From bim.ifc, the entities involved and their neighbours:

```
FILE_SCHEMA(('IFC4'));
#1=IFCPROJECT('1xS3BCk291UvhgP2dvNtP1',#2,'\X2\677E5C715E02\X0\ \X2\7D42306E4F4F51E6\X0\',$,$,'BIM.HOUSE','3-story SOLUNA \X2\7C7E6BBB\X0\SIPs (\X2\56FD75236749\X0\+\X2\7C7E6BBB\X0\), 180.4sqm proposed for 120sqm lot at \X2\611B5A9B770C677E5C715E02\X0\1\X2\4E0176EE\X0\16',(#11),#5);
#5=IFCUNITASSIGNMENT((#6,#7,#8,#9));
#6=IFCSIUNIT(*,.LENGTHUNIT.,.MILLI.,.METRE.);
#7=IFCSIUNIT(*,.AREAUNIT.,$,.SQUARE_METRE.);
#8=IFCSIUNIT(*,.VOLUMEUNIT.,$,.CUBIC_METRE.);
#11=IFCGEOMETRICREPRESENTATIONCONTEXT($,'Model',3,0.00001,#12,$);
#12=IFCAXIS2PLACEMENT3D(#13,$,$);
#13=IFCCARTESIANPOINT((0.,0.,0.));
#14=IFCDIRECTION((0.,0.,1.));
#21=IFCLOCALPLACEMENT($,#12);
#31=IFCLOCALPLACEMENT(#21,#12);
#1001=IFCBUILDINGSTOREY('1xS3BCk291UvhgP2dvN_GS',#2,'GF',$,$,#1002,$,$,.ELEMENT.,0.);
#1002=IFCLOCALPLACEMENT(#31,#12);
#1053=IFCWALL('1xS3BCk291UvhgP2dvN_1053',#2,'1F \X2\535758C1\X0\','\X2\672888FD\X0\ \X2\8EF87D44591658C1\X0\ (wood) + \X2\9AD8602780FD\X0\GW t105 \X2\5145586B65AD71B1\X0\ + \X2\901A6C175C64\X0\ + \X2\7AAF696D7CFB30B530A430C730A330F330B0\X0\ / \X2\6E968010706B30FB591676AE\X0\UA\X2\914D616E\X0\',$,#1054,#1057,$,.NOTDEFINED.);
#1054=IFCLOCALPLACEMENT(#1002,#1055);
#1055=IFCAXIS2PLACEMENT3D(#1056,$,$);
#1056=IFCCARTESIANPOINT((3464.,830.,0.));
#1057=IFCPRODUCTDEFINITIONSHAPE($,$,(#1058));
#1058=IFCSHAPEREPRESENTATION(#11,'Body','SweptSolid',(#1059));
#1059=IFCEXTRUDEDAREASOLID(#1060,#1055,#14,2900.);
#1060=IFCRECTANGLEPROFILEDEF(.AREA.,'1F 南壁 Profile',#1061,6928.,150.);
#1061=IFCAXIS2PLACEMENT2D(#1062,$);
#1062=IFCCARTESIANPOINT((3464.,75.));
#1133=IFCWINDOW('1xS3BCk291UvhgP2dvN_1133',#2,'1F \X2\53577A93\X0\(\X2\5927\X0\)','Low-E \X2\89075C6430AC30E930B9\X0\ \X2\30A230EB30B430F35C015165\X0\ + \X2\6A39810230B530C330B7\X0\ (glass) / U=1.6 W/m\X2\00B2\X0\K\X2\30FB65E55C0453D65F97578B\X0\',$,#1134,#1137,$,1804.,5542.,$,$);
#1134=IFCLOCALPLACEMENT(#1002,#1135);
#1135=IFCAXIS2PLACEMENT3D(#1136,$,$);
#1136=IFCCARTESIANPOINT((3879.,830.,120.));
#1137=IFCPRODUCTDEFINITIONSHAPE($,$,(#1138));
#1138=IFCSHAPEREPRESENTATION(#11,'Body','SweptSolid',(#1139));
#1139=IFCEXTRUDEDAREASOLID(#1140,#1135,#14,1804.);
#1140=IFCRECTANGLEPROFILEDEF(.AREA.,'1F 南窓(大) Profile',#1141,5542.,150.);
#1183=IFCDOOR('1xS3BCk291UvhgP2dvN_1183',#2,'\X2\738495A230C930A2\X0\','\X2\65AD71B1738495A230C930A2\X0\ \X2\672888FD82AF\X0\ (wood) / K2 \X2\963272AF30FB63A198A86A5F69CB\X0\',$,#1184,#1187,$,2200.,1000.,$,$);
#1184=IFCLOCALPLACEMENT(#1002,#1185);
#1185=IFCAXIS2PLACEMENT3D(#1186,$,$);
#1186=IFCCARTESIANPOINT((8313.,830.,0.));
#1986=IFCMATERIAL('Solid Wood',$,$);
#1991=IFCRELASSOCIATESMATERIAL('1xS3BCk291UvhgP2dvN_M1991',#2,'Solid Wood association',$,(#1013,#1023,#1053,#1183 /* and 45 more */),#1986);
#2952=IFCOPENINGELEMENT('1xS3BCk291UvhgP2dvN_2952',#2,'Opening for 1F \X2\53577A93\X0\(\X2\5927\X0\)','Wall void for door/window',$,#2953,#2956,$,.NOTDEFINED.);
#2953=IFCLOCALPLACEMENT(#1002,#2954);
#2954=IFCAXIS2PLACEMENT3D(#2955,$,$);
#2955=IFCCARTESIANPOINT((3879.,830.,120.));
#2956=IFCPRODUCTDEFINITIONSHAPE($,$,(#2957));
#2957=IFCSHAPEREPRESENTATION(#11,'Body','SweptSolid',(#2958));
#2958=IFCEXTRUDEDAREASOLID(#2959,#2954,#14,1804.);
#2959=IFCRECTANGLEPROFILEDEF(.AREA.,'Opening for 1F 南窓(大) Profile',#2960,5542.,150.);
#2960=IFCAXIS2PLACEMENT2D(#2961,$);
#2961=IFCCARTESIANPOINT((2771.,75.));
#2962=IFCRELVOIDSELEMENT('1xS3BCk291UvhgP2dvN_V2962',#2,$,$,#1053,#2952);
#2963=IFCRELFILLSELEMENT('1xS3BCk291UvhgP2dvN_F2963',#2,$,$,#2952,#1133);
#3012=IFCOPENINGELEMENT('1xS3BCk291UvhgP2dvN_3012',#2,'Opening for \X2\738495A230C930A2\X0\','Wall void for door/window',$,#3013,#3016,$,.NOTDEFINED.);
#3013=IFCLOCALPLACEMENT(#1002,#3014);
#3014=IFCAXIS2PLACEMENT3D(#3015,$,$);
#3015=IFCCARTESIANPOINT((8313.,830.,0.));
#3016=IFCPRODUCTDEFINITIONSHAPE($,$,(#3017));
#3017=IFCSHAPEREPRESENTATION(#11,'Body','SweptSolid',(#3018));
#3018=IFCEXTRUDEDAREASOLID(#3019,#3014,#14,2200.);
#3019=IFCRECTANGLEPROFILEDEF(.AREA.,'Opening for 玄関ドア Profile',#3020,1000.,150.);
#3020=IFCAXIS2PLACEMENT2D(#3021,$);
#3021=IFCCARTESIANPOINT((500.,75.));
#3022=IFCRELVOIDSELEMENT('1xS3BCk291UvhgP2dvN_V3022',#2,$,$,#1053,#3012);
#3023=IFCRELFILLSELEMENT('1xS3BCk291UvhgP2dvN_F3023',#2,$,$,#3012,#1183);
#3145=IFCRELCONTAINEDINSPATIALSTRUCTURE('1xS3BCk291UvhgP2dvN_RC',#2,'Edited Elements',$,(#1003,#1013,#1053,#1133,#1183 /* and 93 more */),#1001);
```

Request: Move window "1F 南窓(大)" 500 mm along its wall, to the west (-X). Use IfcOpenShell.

```python
import ifcopenshell
import ifcopenshell.api.geometry
import ifcopenshell.util.placement
import ifcopenshell.util.unit

model = ifcopenshell.open("bim.ifc")
unit_scale = ifcopenshell.util.unit.calculate_unit_scale(model)

window = model.by_guid("1xS3BCk291UvhgP2dvN_1133")
opening = window.FillsVoids[0].RelatingOpeningElement
wall = opening.VoidsElements[0].RelatingBuildingElement

wall_matrix = ifcopenshell.util.placement.get_local_placement(wall.ObjectPlacement)
shift = wall_matrix[:3, 0] * -0.5 / unit_scale
before = ifcopenshell.util.placement.get_local_placement(window.ObjectPlacement)[:3, 3].copy()

# The window is not placed relative to its opening, so move both.
for product in (opening, window):
    matrix = ifcopenshell.util.placement.get_local_placement(product.ObjectPlacement)
    matrix[:3, 3] += shift
    ifcopenshell.api.geometry.edit_object_placement(model, product=product, matrix=matrix, is_si=False)

after = ifcopenshell.util.placement.get_local_placement(window.ObjectPlacement)[:3, 3]
print("window moved by", (after - before).round(3) + 0.0)

model.write("bim-out.ifc")
```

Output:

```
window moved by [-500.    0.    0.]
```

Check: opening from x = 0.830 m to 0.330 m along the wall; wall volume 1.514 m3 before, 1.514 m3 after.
